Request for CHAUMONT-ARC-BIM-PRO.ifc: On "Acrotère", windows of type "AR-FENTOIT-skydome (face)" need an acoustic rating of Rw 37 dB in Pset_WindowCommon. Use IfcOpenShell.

First a look at what the model holds.

```python
import ifcopenshell
import ifcopenshell.util.element

model = ifcopenshell.open("CHAUMONT-ARC-BIM-PRO.ifc")
print(model.schema)
storey = next(s for s in model.by_type("IfcBuildingStorey") if s.Name == "Acrotère")
windows = [e for e in ifcopenshell.util.element.get_decomposition(storey) if e.is_a("IfcWindow")]
seen = {}
for e in windows:
    element_type = ifcopenshell.util.element.get_type(e)
    key = (element_type.Name if element_type != e and element_type else None, ifcopenshell.util.element.get_pset(e, "Pset_WindowCommon", "AcousticRating"))
    seen[key] = seen.get(key, 0) + 1
for (name, value), count in sorted(seen.items(), key=str):
    print(count, "x", name, "|", value)
```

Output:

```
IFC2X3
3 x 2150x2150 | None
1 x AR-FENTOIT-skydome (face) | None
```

```python
import ifcopenshell
import ifcopenshell.api.pset
import ifcopenshell.util.element

model = ifcopenshell.open("CHAUMONT-ARC-BIM-PRO.ifc")

storey = next(s for s in model.by_type("IfcBuildingStorey") if s.Name == "Acrotère")
windows = [e for e in ifcopenshell.util.element.get_decomposition(storey) if e.is_a("IfcWindow")]

count = 0
for e in windows:
    element_type = ifcopenshell.util.element.get_type(e)
    if element_type in (None, e) or element_type.Name != "AR-FENTOIT-skydome (face)":
        continue
    # add_pset returns the element's existing set when there is one.
    pset = ifcopenshell.api.pset.add_pset(model, product=e, name="Pset_WindowCommon")
    ifcopenshell.api.pset.edit_pset(model, pset=pset, properties={"AcousticRating": "Rw 37 dB"})
    count += 1

print(count, "windows updated")

model.write("CHAUMONT-ARC-BIM-PRO_edited.ifc")
```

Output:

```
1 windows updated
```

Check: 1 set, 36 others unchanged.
